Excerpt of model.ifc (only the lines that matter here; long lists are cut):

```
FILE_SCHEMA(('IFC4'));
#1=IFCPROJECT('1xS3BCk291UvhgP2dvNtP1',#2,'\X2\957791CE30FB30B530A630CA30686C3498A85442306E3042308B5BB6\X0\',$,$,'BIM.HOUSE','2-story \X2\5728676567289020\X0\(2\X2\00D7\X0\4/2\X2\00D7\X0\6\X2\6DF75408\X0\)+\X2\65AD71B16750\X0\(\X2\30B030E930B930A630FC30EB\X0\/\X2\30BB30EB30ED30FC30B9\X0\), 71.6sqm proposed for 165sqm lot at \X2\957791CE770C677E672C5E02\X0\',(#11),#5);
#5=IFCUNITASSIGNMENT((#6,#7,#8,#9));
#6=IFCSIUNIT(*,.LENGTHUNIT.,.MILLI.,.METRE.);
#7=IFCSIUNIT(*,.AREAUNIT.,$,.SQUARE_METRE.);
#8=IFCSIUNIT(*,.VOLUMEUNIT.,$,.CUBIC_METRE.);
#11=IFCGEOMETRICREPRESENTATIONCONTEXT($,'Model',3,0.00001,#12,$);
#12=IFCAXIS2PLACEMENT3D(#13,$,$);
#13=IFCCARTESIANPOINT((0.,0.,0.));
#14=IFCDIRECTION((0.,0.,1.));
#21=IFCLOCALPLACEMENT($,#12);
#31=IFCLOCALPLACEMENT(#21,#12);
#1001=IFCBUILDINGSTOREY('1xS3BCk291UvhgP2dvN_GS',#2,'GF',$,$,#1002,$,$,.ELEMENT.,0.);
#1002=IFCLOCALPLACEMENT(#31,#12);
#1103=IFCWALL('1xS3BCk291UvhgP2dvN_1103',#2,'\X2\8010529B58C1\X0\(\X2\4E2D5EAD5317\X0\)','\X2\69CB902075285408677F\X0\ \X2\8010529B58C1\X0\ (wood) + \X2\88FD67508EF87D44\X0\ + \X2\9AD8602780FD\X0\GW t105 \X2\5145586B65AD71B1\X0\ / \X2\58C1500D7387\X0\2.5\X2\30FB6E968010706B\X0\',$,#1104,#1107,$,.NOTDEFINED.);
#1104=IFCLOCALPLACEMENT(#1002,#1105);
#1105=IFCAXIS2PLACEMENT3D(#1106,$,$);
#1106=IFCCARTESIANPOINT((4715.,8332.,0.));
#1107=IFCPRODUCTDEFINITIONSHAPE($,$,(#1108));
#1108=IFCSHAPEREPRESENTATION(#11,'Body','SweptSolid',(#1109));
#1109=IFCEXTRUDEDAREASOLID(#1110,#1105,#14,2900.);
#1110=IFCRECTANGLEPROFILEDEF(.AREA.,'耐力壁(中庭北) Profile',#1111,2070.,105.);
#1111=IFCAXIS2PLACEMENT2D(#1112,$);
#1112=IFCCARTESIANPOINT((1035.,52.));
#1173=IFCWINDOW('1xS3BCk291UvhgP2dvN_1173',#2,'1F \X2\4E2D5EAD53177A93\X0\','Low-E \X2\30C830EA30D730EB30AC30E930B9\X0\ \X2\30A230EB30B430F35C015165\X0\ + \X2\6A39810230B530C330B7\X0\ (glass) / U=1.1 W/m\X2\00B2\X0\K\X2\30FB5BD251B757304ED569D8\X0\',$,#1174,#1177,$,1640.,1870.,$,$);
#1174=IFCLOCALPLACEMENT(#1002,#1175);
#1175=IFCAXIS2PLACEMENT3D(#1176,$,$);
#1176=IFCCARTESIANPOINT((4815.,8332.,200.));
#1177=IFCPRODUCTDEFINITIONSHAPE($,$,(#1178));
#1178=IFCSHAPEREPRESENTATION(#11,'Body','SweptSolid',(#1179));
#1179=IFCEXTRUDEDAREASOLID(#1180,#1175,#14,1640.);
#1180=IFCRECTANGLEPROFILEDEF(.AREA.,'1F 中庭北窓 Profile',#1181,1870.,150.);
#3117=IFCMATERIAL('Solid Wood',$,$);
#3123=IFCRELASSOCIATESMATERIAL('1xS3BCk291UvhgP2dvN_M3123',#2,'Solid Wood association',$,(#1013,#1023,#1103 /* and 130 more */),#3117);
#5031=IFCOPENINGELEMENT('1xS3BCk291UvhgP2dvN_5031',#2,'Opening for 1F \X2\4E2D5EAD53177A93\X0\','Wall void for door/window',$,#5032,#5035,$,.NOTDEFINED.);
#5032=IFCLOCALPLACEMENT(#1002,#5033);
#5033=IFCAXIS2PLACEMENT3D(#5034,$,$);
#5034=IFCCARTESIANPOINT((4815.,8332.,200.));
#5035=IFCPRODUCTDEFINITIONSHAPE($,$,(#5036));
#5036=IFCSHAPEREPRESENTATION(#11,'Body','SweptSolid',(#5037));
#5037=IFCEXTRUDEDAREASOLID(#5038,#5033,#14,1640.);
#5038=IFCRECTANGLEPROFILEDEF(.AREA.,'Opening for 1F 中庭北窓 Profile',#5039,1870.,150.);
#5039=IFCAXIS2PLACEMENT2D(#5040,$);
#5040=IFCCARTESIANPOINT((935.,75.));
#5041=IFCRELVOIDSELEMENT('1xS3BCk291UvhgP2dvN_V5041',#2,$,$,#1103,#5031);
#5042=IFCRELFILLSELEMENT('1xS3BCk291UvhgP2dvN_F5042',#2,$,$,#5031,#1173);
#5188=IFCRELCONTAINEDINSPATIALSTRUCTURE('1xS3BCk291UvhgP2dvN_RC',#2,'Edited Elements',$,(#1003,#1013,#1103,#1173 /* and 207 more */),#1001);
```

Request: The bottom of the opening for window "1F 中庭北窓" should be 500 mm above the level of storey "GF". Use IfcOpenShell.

```python
import numpy as np
import ifcopenshell
import ifcopenshell.api.geometry
import ifcopenshell.geom
import ifcopenshell.util.element
import ifcopenshell.util.placement
import ifcopenshell.util.shape
import ifcopenshell.util.unit

model = ifcopenshell.open("model.ifc")
unit_scale = ifcopenshell.util.unit.calculate_unit_scale(model)

window = model.by_guid("1xS3BCk291UvhgP2dvN_1173")
opening = window.FillsVoids[0].RelatingOpeningElement
storey = ifcopenshell.util.element.get_container(window, ifc_class="IfcBuildingStorey")
level = ifcopenshell.util.placement.get_local_placement(storey.ObjectPlacement)[2, 3]

# The opening's origin need not be at the sill, so measure its lowest point.
shape = ifcopenshell.geom.create_shape(ifcopenshell.geom.settings(), opening)
bottom = ifcopenshell.util.shape.get_shape_bottom_elevation(shape, shape.geometry) / unit_scale
dz = level + 0.5 / unit_scale - bottom

shift = np.array([0.0, 0.0, dz])
# The window is not placed relative to its opening, so move both.
for product in (opening, window):
    matrix = ifcopenshell.util.placement.get_local_placement(product.ObjectPlacement)
    matrix[:3, 3] += shift
    ifcopenshell.api.geometry.edit_object_placement(model, product=product, matrix=matrix, is_si=False)

print(f"moved by {dz * unit_scale:+.3f} m")

model.write("model_edited.ifc")
```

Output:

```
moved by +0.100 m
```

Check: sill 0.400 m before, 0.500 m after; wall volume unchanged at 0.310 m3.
